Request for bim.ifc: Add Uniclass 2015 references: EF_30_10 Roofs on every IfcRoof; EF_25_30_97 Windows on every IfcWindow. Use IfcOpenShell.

First a look at what the model holds.

```python
import ifcopenshell

model = ifcopenshell.open("bim.ifc")
print(model.schema)
print("classifications:", [c.Name for c in model.by_type("IfcClassification")])
for ifc_class in ("IfcDoor", "IfcRoof", "IfcStair", "IfcWall", "IfcWindow"):
    print(ifc_class, len(model.by_type(ifc_class)))
```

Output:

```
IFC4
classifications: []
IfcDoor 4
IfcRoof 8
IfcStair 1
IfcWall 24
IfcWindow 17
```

```python
import ifcopenshell
import ifcopenshell.api.classification

model = ifcopenshell.open("bim.ifc")

system = ifcopenshell.api.classification.add_classification(model, classification="Uniclass 2015")

codes = {
    "IfcRoof": ("EF_30_10", "Roofs"),
    "IfcWindow": ("EF_25_30_97", "Windows"),
}
for ifc_class, (code, name) in codes.items():
    products = model.by_type(ifc_class)
    ifcopenshell.api.classification.add_reference(
        model, products=products, classification=system, identification=code, name=name
    )
    print(code, len(products))

model.write("bim_v2.ifc")
```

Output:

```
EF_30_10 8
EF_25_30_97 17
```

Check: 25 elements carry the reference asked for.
